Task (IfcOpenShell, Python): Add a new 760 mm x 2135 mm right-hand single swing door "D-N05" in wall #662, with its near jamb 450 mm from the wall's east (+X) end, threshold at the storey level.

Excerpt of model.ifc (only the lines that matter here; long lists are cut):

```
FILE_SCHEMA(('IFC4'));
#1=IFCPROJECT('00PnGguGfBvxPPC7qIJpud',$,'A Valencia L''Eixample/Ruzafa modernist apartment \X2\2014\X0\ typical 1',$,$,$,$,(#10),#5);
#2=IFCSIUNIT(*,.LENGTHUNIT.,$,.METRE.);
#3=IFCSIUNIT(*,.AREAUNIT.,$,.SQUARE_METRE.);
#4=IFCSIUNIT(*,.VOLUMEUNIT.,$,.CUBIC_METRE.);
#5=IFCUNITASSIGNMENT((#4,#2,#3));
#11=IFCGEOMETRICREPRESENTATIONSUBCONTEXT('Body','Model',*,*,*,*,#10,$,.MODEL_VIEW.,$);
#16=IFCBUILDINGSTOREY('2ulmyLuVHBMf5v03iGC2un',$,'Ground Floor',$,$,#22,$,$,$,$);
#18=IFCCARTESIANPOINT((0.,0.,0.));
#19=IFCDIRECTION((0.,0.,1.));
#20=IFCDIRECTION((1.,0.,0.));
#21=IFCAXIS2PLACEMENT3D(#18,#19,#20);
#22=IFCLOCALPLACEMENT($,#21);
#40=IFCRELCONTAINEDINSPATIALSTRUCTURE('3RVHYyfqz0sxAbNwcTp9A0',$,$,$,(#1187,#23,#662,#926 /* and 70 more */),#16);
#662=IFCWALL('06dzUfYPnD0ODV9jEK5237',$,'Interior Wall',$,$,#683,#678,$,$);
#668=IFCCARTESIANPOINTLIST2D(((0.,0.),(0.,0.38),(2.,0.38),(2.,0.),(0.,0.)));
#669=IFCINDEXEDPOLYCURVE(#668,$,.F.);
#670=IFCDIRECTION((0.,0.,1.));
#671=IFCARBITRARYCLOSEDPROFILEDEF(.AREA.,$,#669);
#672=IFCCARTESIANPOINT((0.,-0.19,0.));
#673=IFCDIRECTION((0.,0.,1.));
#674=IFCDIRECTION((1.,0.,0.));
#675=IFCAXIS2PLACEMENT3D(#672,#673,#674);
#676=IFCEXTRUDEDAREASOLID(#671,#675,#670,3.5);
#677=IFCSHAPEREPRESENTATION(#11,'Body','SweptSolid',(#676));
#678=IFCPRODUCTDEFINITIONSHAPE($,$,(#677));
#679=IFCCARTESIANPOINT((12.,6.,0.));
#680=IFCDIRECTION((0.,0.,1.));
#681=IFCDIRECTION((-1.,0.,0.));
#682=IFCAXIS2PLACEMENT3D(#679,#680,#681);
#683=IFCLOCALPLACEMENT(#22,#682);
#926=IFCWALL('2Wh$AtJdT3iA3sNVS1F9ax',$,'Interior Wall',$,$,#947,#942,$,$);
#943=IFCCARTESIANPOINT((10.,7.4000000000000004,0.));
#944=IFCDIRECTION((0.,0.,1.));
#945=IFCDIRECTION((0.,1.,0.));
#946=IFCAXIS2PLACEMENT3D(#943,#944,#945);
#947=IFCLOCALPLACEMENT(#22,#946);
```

```python
import numpy as np
import ifcopenshell
import ifcopenshell.api.feature
import ifcopenshell.api.geometry
import ifcopenshell.api.root
import ifcopenshell.api.spatial
import ifcopenshell.geom
import ifcopenshell.util.element
import ifcopenshell.util.placement
import ifcopenshell.util.representation
import ifcopenshell.util.shape
import ifcopenshell.util.unit

model = ifcopenshell.open("model.ifc")
unit_scale = ifcopenshell.util.unit.calculate_unit_scale(model)
settings = ifcopenshell.geom.settings()


def volume(element):
    """Net volume in cubic metres, openings subtracted."""
    shape = ifcopenshell.geom.create_shape(settings, element)
    return ifcopenshell.util.shape.get_volume(shape.geometry)


wall = model.by_id(662)
storey = ifcopenshell.util.element.get_container(wall, ifc_class="IfcBuildingStorey")
context = ifcopenshell.util.representation.get_context(model, "Model", "Body", "MODEL_VIEW")
before = volume(wall)

width, height, from_end, sill = 0.76, 2.135, 0.45, 0.0  # metres

# The wall runs along its own X axis, and the end named is its -X end.
wall_shape = ifcopenshell.geom.create_shape(settings, wall)
x, y, z = ifcopenshell.util.shape.get_vertices(wall_shape.geometry).T
start = x.min() + from_end
face, thickness = float(y.min()), float(y.max() - y.min())
wall_matrix = ifcopenshell.util.placement.get_local_placement(wall.ObjectPlacement)
level = ifcopenshell.util.placement.get_local_placement(storey.ObjectPlacement)[2, 3]


def in_wall(x, y):
    """Placement at x, y metres in the wall's axes, at sill height."""
    matrix = wall_matrix.copy()
    matrix[:, 3] = wall_matrix @ np.array([x / unit_scale, y / unit_scale, 0.0, 1.0])
    matrix[2, 3] = level + sill / unit_scale
    return matrix


# Opening: a box that overshoots both wall faces by 50 mm.
opening = ifcopenshell.api.root.create_entity(model, ifc_class="IfcOpeningElement", predefined_type="OPENING")
box = ifcopenshell.api.geometry.add_wall_representation(
    model, context=context, length=width, height=height, thickness=thickness + 0.1
)
ifcopenshell.api.geometry.assign_representation(model, product=opening, representation=box)
ifcopenshell.api.geometry.edit_object_placement(model, product=opening, matrix=in_wall(start, face - 0.05), is_si=False)
ifcopenshell.api.feature.add_feature(model, feature=opening, element=wall)

door = ifcopenshell.api.root.create_entity(model, ifc_class="IfcDoor", name="D-N05", predefined_type="DOOR")
door.OverallWidth, door.OverallHeight = width / unit_scale, height / unit_scale
door.OperationType = "SINGLE_SWING_RIGHT"
body = ifcopenshell.api.geometry.add_door_representation(
    model,
    context=context,
    overall_width=door.OverallWidth,
    overall_height=door.OverallHeight,
    operation_type="SINGLE_SWING_RIGHT",
    lining_properties={"LiningDepth": thickness / unit_scale, "ThresholdDepth": thickness / unit_scale},
)
ifcopenshell.api.geometry.assign_representation(model, product=door, representation=body)
ifcopenshell.api.spatial.assign_container(model, products=[door], relating_structure=storey)
ifcopenshell.api.feature.add_filling(model, opening=opening, element=door)

# The lining spans the wall, so the door starts at the wall face.
ifcopenshell.api.geometry.edit_object_placement(model, product=door, matrix=in_wall(start, face), is_si=False)

after = volume(wall)

print(f"wall volume {before:.3f} -> {after:.3f} m3")

model.write("model-out.ifc")
```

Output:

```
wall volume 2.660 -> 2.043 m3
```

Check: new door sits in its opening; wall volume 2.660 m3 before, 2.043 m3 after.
